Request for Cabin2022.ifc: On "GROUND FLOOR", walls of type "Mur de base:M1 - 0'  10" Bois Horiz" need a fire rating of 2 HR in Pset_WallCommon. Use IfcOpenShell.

First a look at what the model holds.

```python
import ifcopenshell
import ifcopenshell.util.element

model = ifcopenshell.open("Cabin2022.ifc")
print(model.schema)
storey = next(s for s in model.by_type("IfcBuildingStorey") if s.Name == "GROUND FLOOR")
walls = [e for e in ifcopenshell.util.element.get_decomposition(storey) if e.is_a("IfcWall")]
seen = {}
for e in walls:
    element_type = ifcopenshell.util.element.get_type(e)
    key = (element_type.Name if element_type != e and element_type else None, ifcopenshell.util.element.get_pset(e, "Pset_WallCommon", "FireRating"))
    seen[key] = seen.get(key, 0) + 1
for (name, value), count in sorted(seen.items(), key=str):
    print(count, "x", name, "|", value)
```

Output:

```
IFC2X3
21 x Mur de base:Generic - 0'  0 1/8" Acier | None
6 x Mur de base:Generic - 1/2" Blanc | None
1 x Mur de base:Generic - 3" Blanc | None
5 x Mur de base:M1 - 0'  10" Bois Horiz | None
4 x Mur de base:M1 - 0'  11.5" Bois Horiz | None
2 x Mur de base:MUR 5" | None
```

```python
import ifcopenshell
import ifcopenshell.api.pset
import ifcopenshell.util.element

model = ifcopenshell.open("Cabin2022.ifc")

storey = next(s for s in model.by_type("IfcBuildingStorey") if s.Name == "GROUND FLOOR")
walls = [e for e in ifcopenshell.util.element.get_decomposition(storey) if e.is_a("IfcWall")]

count = 0
for e in walls:
    element_type = ifcopenshell.util.element.get_type(e)
    if element_type in (None, e) or element_type.Name != 'Mur de base:M1 - 0\'  10" Bois Horiz':
        continue
    # add_pset returns the element's existing set when there is one.
    pset = ifcopenshell.api.pset.add_pset(model, product=e, name="Pset_WallCommon")
    ifcopenshell.api.pset.edit_pset(model, pset=pset, properties={"FireRating": "2 HR"})
    count += 1

print(count, "walls updated")

model.write("Cabin2022_v2.ifc")
```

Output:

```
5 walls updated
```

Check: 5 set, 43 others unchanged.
